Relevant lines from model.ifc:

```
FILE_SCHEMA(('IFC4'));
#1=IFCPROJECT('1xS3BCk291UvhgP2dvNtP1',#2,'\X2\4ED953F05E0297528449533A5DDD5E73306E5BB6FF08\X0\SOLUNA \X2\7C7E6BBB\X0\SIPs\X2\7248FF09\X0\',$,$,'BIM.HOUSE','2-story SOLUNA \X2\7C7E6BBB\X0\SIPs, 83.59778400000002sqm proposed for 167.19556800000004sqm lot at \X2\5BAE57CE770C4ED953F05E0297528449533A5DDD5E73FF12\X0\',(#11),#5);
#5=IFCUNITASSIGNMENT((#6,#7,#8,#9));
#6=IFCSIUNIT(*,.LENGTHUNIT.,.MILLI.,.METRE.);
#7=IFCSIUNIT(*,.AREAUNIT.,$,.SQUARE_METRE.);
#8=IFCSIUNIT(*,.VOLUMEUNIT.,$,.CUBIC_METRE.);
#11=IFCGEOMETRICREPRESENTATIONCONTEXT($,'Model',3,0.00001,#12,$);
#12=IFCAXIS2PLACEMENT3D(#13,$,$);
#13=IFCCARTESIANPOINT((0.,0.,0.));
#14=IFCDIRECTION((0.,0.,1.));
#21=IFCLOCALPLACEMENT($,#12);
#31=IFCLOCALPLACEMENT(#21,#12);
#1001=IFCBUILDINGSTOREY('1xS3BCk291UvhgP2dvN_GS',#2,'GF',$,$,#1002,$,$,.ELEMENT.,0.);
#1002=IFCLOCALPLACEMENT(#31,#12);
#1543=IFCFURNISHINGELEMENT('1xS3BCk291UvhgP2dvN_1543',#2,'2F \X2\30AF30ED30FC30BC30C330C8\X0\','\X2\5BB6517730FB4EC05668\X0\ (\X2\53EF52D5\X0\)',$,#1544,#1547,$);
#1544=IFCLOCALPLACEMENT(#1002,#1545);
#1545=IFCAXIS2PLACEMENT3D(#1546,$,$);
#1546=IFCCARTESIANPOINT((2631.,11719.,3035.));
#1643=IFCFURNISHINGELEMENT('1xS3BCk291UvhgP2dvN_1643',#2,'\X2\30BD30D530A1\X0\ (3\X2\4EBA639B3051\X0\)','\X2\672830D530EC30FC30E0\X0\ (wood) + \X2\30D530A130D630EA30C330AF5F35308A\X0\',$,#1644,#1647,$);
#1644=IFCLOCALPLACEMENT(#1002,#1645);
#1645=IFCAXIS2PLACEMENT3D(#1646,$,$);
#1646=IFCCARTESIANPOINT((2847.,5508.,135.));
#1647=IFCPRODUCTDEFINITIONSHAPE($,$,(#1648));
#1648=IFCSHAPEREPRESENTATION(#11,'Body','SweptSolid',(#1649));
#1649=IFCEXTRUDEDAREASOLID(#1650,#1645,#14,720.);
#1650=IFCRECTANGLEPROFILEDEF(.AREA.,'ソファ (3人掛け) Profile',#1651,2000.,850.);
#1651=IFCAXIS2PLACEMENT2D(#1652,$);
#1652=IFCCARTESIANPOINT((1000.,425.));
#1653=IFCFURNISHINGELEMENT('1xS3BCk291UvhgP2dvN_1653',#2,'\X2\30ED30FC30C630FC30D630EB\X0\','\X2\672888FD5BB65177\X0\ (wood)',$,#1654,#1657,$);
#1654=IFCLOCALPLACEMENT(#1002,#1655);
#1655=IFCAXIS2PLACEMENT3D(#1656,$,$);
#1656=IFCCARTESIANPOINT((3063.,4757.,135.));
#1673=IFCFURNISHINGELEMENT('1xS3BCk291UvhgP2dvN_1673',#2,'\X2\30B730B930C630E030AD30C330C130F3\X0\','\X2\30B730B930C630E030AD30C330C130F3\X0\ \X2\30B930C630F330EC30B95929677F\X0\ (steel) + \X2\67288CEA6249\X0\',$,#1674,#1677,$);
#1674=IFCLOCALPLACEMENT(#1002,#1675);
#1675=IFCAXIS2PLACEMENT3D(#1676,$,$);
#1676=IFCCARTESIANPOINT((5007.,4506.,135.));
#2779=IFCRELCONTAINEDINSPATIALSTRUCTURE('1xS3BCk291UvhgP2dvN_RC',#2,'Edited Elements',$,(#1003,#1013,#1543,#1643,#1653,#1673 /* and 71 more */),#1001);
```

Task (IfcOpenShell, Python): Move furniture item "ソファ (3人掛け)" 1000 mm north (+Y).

```python
import ifcopenshell
import ifcopenshell.api.geometry
import ifcopenshell.util.placement

model = ifcopenshell.open("model.ifc")

item = model.by_id(1643)
matrix = ifcopenshell.util.placement.get_local_placement(item.ObjectPlacement)
matrix[1, 3] += 1000.0
ifcopenshell.api.geometry.edit_object_placement(model, product=item, matrix=matrix, is_si=False)

print(ifcopenshell.util.placement.get_local_placement(item.ObjectPlacement).round(3) + 0.0)

model.write("model_rev.ifc")
```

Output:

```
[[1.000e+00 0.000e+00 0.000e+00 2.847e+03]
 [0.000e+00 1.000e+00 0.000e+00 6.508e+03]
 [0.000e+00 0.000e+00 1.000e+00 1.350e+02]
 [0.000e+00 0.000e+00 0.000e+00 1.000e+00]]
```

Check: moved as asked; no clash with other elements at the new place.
